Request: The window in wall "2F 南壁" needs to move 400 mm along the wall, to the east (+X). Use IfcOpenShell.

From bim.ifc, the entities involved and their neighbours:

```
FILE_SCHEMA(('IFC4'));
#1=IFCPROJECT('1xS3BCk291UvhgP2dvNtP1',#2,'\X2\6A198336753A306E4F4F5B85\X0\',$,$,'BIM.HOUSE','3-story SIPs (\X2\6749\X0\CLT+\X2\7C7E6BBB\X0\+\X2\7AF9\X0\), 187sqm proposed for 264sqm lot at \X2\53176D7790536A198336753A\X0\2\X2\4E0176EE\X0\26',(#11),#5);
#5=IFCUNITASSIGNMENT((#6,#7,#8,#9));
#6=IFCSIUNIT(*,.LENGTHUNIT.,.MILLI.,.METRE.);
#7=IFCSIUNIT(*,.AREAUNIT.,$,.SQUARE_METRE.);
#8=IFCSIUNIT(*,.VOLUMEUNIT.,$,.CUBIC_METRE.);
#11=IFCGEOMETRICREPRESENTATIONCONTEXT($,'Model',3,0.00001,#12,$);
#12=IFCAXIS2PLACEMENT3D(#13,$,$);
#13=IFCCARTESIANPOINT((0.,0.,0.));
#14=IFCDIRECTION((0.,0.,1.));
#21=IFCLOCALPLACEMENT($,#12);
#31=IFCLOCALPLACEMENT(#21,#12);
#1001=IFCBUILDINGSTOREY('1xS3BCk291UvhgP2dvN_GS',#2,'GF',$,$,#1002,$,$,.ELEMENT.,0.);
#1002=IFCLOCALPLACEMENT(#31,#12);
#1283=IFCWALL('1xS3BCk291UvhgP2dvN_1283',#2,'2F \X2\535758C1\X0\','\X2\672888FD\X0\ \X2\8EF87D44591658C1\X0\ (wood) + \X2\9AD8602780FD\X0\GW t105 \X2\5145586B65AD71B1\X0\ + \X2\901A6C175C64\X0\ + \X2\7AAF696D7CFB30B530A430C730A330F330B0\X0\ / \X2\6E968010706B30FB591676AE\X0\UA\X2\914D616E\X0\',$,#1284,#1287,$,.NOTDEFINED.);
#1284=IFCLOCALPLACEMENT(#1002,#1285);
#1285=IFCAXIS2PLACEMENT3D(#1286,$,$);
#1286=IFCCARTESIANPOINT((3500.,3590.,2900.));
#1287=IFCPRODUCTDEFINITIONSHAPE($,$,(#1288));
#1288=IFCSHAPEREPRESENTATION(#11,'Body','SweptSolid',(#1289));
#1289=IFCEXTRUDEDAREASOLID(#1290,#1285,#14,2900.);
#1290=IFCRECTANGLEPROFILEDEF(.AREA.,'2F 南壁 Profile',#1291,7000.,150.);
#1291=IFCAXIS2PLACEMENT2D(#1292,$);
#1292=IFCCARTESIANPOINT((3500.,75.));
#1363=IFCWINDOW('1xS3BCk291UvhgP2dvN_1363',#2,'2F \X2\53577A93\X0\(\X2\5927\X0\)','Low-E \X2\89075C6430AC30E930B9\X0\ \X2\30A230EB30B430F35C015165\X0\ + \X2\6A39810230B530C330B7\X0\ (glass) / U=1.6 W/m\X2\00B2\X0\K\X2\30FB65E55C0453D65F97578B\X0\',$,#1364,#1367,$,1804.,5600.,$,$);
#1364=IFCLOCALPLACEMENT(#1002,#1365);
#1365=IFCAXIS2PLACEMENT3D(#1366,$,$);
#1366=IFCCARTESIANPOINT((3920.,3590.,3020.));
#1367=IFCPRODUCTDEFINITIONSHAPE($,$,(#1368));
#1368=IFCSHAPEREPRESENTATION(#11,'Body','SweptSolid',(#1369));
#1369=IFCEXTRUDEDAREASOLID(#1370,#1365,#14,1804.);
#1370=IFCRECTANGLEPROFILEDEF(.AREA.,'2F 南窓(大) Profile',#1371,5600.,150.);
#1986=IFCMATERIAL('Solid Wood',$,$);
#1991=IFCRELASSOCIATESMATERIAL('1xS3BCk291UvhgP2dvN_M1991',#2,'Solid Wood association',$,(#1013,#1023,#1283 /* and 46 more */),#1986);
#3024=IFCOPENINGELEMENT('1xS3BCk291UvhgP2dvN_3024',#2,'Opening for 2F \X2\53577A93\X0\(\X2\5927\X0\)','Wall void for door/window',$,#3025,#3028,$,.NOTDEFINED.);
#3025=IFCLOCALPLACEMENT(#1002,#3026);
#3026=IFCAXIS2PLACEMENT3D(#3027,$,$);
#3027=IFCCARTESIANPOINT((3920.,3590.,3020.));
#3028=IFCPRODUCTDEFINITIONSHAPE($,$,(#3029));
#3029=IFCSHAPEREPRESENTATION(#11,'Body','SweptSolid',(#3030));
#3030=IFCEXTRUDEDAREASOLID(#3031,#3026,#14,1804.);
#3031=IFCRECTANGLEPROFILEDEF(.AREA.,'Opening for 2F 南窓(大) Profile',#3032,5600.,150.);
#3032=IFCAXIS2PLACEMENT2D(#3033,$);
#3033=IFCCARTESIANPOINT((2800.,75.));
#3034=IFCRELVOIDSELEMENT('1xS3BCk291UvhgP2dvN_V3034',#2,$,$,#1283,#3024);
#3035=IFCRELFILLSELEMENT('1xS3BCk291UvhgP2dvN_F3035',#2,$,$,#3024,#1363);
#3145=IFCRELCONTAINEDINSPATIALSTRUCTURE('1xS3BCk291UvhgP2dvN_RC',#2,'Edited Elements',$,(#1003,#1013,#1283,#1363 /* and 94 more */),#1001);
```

```python
import ifcopenshell
import ifcopenshell.api.geometry
import ifcopenshell.util.placement
import ifcopenshell.util.unit

model = ifcopenshell.open("bim.ifc")
unit_scale = ifcopenshell.util.unit.calculate_unit_scale(model)

window = model.by_guid("1xS3BCk291UvhgP2dvN_1363")
opening = window.FillsVoids[0].RelatingOpeningElement
wall = opening.VoidsElements[0].RelatingBuildingElement

wall_matrix = ifcopenshell.util.placement.get_local_placement(wall.ObjectPlacement)
shift = wall_matrix[:3, 0] * 0.4 / unit_scale
before = ifcopenshell.util.placement.get_local_placement(window.ObjectPlacement)[:3, 3].copy()

# The window is not placed relative to its opening, so move both.
for product in (opening, window):
    matrix = ifcopenshell.util.placement.get_local_placement(product.ObjectPlacement)
    matrix[:3, 3] += shift
    ifcopenshell.api.geometry.edit_object_placement(model, product=product, matrix=matrix, is_si=False)

after = ifcopenshell.util.placement.get_local_placement(window.ObjectPlacement)[:3, 3]
print("window moved by", (after - before).round(3) + 0.0)

model.write("bim_edited.ifc")
```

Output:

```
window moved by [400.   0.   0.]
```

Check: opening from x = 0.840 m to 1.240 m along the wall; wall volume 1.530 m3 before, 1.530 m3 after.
